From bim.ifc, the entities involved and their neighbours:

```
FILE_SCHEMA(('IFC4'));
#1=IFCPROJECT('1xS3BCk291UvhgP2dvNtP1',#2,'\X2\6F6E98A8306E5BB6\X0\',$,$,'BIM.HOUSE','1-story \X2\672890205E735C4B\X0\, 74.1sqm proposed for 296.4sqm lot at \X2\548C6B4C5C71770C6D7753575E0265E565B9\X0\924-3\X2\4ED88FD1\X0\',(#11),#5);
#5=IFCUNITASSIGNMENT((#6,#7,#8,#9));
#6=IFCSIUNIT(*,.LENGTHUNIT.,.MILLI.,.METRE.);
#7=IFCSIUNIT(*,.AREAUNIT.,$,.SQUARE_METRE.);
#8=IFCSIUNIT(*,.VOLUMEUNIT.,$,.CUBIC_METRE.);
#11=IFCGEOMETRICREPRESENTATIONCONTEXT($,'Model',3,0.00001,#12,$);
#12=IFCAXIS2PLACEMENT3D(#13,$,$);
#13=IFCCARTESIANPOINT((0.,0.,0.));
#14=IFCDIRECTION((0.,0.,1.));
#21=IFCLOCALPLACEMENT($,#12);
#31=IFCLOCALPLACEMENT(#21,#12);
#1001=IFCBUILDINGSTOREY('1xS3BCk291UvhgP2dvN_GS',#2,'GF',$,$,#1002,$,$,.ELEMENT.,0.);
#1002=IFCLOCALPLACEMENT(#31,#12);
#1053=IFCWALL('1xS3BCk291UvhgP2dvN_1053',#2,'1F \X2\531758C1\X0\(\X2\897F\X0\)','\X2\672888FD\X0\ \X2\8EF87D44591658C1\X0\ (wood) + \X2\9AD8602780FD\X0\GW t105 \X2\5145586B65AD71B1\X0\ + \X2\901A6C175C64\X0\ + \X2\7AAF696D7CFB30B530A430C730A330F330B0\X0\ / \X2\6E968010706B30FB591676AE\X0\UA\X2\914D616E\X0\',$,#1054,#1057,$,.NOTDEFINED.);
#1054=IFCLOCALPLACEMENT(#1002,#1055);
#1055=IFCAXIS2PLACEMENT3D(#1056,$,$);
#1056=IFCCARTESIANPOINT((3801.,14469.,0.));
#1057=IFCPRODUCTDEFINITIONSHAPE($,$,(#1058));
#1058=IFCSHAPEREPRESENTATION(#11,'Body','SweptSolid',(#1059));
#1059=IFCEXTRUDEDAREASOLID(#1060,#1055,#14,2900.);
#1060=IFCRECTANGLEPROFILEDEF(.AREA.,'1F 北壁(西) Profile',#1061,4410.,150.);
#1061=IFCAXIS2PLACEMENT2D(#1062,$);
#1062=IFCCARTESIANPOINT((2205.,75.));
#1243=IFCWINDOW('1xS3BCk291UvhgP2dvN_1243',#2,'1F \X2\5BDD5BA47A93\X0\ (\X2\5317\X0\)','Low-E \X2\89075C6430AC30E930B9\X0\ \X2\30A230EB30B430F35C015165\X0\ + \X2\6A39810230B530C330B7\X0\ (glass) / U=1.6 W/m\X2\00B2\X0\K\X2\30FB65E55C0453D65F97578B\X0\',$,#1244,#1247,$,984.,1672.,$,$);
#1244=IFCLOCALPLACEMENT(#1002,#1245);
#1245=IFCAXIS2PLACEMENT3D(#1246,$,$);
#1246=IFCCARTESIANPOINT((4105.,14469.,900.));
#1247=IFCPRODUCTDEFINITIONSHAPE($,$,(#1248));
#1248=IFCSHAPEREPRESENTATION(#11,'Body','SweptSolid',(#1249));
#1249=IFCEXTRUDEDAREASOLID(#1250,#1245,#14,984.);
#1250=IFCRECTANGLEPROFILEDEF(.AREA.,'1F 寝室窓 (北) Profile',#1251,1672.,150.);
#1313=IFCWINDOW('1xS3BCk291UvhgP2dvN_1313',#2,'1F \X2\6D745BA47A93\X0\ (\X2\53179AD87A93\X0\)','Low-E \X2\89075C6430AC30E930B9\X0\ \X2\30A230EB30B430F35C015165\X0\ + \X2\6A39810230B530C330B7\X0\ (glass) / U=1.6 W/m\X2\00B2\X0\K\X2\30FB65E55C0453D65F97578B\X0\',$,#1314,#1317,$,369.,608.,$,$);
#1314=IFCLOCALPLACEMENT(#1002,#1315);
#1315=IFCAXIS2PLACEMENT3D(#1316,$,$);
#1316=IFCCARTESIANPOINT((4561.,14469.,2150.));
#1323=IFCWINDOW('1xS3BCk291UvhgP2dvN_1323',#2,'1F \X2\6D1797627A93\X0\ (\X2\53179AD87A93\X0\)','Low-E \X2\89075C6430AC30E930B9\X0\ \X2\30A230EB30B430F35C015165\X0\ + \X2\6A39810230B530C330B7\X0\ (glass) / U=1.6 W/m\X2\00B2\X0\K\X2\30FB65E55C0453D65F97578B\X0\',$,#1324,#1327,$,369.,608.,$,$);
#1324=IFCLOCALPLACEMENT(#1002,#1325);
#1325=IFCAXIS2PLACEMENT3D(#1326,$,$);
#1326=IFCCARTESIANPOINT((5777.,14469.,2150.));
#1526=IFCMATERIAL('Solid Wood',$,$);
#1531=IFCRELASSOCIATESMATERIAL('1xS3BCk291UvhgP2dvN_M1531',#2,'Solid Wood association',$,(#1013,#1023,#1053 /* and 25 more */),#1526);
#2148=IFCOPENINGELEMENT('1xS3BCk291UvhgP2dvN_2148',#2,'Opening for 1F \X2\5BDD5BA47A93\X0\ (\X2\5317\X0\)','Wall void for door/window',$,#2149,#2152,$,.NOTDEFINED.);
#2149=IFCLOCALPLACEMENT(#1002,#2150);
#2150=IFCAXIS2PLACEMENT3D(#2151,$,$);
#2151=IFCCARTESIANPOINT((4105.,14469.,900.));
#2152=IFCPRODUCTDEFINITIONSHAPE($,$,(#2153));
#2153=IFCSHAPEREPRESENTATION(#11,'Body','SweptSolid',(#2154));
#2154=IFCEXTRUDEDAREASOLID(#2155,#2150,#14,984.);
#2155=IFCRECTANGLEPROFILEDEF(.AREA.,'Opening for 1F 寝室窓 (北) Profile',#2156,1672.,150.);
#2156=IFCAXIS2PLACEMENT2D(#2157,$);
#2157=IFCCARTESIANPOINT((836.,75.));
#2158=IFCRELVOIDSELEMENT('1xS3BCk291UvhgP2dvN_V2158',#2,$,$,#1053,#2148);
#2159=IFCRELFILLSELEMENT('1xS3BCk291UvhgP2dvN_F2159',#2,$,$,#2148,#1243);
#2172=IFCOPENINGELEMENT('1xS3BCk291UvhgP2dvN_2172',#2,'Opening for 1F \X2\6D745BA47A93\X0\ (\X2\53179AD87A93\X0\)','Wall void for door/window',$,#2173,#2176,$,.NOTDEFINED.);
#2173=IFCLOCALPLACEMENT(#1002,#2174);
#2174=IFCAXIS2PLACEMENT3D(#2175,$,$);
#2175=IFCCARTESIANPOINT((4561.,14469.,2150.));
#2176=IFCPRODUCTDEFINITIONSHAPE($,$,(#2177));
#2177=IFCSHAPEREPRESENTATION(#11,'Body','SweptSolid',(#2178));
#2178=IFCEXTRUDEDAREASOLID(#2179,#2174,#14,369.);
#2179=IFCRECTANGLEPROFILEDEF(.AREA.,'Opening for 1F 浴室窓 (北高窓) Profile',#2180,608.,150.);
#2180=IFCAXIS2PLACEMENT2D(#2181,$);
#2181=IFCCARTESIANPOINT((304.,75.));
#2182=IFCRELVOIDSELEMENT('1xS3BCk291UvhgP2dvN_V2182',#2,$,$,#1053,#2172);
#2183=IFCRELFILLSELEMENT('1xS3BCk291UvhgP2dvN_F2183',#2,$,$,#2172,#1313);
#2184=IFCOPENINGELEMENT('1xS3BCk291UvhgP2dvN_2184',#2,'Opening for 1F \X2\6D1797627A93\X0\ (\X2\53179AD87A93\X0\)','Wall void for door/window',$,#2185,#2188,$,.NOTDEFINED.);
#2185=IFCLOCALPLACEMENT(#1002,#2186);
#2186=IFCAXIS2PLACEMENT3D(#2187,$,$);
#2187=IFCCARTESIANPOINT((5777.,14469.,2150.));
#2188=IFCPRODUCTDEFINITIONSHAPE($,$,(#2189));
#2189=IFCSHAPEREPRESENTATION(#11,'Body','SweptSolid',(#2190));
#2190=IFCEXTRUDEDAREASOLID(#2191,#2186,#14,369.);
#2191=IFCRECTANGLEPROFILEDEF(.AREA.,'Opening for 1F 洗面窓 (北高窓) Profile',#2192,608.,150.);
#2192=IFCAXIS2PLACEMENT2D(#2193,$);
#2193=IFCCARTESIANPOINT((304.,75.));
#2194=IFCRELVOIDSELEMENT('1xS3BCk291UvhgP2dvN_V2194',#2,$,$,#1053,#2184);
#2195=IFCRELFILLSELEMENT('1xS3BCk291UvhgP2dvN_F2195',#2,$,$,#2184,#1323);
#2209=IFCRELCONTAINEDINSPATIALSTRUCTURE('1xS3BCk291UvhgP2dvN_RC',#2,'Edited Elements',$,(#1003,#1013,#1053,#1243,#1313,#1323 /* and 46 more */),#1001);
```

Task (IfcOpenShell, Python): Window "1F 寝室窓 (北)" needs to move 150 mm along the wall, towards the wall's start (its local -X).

```python
import ifcopenshell
import ifcopenshell.api.geometry
import ifcopenshell.util.placement
import ifcopenshell.util.unit

model = ifcopenshell.open("bim.ifc")
unit_scale = ifcopenshell.util.unit.calculate_unit_scale(model)

window = model.by_guid("1xS3BCk291UvhgP2dvN_1243")
opening = window.FillsVoids[0].RelatingOpeningElement
wall = opening.VoidsElements[0].RelatingBuildingElement

wall_matrix = ifcopenshell.util.placement.get_local_placement(wall.ObjectPlacement)
shift = wall_matrix[:3, 0] * -0.15 / unit_scale
before = ifcopenshell.util.placement.get_local_placement(window.ObjectPlacement)[:3, 3].copy()

# The window is not placed relative to its opening, so move both.
for product in (opening, window):
    matrix = ifcopenshell.util.placement.get_local_placement(product.ObjectPlacement)
    matrix[:3, 3] += shift
    ifcopenshell.api.geometry.edit_object_placement(model, product=product, matrix=matrix, is_si=False)

after = ifcopenshell.util.placement.get_local_placement(window.ObjectPlacement)[:3, 3]
print("window moved by", (after - before).round(3) + 0.0)

model.write("bim_updated.ifc")
```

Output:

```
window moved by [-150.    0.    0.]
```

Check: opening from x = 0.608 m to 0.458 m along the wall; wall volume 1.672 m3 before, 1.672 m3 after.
